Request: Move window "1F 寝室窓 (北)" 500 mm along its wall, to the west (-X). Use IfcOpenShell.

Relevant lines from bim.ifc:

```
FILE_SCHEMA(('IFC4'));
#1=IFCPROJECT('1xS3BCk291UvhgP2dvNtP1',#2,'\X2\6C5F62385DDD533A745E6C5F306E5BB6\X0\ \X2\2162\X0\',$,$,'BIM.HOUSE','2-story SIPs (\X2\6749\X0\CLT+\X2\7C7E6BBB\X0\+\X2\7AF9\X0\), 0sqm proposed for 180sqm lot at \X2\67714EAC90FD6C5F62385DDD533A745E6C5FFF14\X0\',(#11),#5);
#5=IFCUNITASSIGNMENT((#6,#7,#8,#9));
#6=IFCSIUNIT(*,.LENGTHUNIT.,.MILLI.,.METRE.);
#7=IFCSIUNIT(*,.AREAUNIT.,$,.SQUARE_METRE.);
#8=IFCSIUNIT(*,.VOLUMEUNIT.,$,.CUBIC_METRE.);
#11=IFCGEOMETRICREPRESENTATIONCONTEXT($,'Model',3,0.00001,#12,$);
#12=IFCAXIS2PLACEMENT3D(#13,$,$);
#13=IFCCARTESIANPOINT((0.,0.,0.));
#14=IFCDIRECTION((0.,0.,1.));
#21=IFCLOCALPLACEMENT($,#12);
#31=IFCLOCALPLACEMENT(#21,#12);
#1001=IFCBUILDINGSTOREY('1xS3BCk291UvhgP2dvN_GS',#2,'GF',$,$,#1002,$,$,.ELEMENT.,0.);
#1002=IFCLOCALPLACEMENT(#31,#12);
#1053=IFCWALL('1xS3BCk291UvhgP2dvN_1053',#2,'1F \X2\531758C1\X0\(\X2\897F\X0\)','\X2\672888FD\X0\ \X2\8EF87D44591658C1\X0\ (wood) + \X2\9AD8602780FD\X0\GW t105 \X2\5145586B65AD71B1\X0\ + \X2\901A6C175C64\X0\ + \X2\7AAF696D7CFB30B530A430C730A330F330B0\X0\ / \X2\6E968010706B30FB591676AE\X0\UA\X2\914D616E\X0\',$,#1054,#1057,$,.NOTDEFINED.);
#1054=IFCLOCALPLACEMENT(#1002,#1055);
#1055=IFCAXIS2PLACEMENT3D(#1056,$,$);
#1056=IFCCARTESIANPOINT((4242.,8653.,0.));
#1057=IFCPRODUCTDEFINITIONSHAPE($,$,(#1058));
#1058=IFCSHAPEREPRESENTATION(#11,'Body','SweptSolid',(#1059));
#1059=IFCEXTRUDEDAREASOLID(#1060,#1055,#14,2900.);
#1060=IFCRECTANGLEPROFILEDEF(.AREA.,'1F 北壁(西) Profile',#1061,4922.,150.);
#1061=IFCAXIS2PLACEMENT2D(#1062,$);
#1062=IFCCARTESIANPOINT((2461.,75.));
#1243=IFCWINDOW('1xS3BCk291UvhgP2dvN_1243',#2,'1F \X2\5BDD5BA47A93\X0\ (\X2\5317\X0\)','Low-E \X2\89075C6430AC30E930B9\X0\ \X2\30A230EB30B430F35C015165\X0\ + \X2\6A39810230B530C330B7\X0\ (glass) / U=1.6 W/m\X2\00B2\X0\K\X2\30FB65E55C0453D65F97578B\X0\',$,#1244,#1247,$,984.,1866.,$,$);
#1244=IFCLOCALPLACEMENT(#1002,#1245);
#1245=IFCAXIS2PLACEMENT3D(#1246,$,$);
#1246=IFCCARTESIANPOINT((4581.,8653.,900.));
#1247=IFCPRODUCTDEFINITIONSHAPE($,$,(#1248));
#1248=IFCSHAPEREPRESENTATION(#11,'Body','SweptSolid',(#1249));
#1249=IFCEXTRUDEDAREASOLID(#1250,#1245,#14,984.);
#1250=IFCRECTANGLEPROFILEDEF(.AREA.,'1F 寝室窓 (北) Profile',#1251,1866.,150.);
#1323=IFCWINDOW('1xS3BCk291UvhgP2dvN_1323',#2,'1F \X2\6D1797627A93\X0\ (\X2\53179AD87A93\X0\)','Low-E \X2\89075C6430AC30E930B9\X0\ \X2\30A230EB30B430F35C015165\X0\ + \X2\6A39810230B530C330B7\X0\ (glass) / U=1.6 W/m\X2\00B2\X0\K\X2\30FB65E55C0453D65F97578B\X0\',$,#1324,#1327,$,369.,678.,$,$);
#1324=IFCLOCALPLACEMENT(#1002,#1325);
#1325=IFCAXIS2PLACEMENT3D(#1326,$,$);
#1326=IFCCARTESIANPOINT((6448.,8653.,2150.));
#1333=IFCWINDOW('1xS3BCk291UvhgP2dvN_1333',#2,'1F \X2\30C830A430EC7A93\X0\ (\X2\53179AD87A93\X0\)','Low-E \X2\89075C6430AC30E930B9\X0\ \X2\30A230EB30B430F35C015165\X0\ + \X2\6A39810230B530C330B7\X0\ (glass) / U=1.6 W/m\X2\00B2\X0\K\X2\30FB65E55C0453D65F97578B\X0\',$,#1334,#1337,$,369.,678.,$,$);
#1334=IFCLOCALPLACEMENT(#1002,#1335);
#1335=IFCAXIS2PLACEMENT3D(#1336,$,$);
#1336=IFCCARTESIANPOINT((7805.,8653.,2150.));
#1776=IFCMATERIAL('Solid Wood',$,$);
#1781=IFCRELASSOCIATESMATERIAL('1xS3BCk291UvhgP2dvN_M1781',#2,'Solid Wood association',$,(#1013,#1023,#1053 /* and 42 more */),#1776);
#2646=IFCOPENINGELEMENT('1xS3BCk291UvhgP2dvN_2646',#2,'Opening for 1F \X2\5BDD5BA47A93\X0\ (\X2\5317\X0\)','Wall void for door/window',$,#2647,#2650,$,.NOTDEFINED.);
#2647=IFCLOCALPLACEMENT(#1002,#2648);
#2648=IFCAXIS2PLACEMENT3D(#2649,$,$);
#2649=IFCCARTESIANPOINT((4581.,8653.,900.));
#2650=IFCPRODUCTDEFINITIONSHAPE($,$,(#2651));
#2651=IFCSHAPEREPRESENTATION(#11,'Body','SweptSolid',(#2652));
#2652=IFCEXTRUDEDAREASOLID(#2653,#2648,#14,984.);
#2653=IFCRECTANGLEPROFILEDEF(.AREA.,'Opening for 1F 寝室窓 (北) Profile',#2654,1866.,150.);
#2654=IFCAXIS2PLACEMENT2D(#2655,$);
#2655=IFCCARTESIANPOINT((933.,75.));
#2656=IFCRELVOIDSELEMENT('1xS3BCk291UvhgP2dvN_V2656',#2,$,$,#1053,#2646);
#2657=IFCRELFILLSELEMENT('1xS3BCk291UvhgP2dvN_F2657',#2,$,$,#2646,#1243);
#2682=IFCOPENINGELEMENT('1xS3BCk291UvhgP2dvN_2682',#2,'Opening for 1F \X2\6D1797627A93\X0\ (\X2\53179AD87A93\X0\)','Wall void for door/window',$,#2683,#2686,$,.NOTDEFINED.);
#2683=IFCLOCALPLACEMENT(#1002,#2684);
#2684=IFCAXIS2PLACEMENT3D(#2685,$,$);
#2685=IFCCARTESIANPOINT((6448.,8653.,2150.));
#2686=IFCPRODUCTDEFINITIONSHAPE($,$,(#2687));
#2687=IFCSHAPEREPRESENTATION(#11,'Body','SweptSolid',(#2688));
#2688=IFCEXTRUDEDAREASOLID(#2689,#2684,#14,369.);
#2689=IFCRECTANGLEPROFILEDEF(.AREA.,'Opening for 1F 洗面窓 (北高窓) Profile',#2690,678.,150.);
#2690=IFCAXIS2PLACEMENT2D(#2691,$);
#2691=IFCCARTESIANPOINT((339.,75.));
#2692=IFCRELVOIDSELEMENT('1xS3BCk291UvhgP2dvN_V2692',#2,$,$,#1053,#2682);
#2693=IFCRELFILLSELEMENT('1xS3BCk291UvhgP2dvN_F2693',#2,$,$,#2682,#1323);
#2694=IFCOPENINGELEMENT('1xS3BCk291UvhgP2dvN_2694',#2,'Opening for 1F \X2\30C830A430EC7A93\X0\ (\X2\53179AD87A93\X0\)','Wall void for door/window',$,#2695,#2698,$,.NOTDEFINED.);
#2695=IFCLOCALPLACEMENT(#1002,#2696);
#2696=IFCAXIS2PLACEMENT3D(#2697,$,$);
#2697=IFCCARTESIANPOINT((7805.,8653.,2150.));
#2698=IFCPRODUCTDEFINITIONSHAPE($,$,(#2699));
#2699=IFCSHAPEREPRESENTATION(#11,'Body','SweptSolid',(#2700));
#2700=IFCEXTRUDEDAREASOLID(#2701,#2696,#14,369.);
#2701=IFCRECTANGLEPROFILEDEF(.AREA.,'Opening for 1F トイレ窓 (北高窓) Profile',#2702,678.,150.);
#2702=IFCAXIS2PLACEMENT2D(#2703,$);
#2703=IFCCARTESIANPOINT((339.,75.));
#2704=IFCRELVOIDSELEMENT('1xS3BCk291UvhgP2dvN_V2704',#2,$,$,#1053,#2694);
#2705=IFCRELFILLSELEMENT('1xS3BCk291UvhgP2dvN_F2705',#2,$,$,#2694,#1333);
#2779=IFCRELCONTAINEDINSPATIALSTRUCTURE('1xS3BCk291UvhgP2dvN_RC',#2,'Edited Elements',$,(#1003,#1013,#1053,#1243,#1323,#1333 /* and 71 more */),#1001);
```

```python
import ifcopenshell
import ifcopenshell.api.geometry
import ifcopenshell.util.placement
import ifcopenshell.util.unit

model = ifcopenshell.open("bim.ifc")
unit_scale = ifcopenshell.util.unit.calculate_unit_scale(model)

window = model.by_id(1243)
opening = window.FillsVoids[0].RelatingOpeningElement
wall = opening.VoidsElements[0].RelatingBuildingElement

wall_matrix = ifcopenshell.util.placement.get_local_placement(wall.ObjectPlacement)
shift = wall_matrix[:3, 0] * -0.5 / unit_scale
before = ifcopenshell.util.placement.get_local_placement(window.ObjectPlacement)[:3, 3].copy()

# The window is not placed relative to its opening, so move both.
for product in (opening, window):
    matrix = ifcopenshell.util.placement.get_local_placement(product.ObjectPlacement)
    matrix[:3, 3] += shift
    ifcopenshell.api.geometry.edit_object_placement(model, product=product, matrix=matrix, is_si=False)

after = ifcopenshell.util.placement.get_local_placement(window.ObjectPlacement)[:3, 3]
print("window moved by", (after - before).round(3) + 0.0)

model.write("bim_v2.ifc")
```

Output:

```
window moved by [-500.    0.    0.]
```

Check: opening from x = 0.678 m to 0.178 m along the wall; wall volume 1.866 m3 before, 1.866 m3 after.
